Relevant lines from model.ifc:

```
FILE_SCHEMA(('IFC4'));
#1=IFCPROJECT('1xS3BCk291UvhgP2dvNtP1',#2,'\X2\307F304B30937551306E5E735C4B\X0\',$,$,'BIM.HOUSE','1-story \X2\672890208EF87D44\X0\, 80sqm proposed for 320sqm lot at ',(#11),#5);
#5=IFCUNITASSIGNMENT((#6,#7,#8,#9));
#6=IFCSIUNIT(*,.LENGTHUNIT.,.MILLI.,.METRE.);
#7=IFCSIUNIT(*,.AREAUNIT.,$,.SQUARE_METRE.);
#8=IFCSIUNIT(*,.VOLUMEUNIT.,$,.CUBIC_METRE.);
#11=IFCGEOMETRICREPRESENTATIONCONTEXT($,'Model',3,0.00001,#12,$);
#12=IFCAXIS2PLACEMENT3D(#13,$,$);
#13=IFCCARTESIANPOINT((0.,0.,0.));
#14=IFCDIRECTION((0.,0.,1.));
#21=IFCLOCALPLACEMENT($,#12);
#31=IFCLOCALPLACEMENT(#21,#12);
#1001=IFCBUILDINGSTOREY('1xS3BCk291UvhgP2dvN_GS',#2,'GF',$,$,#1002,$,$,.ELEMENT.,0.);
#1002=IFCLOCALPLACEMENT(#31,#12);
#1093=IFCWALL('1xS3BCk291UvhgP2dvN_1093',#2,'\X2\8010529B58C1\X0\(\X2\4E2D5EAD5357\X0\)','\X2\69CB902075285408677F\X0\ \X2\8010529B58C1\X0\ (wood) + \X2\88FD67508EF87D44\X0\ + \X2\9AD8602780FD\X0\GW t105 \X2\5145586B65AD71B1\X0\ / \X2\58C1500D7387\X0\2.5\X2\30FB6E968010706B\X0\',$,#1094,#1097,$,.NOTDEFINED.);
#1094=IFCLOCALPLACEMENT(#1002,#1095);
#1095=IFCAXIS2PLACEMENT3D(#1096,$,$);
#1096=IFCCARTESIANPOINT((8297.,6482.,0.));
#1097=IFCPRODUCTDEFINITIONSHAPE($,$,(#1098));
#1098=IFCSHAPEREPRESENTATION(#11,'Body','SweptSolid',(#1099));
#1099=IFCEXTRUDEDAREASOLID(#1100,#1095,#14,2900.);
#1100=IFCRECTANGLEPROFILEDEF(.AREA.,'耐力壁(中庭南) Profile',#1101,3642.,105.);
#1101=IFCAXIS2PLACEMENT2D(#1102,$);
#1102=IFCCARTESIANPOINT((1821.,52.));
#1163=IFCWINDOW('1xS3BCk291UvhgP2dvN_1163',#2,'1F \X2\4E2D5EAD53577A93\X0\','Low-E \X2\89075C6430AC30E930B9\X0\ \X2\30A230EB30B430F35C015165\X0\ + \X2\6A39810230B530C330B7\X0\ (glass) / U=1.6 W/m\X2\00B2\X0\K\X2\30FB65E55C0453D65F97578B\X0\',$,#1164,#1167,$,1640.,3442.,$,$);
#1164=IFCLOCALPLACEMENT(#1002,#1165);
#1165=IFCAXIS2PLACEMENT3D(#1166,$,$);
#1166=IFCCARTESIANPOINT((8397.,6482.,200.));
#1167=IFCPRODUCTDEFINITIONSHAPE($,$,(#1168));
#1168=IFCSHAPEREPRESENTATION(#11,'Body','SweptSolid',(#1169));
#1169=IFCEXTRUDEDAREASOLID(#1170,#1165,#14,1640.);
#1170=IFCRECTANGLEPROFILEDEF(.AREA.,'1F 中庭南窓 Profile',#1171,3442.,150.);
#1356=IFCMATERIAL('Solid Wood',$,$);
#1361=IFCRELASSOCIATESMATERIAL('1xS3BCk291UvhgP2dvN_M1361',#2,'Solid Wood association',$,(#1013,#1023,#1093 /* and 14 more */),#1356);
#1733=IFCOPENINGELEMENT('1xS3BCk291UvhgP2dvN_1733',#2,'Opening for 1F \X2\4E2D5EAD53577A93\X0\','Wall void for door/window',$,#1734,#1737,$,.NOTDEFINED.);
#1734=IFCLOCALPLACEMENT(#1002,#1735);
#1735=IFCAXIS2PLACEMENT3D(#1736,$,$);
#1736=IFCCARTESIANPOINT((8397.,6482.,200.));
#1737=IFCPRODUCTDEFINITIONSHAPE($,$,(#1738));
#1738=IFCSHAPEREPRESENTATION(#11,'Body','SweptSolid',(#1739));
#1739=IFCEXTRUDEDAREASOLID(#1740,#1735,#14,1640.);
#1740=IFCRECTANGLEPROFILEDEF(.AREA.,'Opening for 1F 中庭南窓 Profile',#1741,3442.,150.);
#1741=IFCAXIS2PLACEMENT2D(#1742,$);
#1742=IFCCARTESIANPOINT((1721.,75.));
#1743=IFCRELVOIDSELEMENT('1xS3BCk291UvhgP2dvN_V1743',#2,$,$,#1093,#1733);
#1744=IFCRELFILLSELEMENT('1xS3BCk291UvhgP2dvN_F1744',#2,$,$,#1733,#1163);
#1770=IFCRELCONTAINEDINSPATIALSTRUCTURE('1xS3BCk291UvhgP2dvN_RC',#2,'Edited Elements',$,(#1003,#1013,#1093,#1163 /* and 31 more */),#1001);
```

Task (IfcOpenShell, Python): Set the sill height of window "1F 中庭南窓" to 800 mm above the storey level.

```python
import numpy as np
import ifcopenshell
import ifcopenshell.api.geometry
import ifcopenshell.geom
import ifcopenshell.util.element
import ifcopenshell.util.placement
import ifcopenshell.util.shape
import ifcopenshell.util.unit

model = ifcopenshell.open("model.ifc")
unit_scale = ifcopenshell.util.unit.calculate_unit_scale(model)

window = model.by_id(1163)
opening = window.FillsVoids[0].RelatingOpeningElement
storey = ifcopenshell.util.element.get_container(window, ifc_class="IfcBuildingStorey")
level = ifcopenshell.util.placement.get_local_placement(storey.ObjectPlacement)[2, 3]

# The opening's origin need not be at the sill, so measure its lowest point.
shape = ifcopenshell.geom.create_shape(ifcopenshell.geom.settings(), opening)
bottom = ifcopenshell.util.shape.get_shape_bottom_elevation(shape, shape.geometry) / unit_scale
dz = level + 800.0 - bottom

shift = np.array([0.0, 0.0, dz])
# The window is not placed relative to its opening, so move both.
for product in (opening, window):
    matrix = ifcopenshell.util.placement.get_local_placement(product.ObjectPlacement)
    matrix[:3, 3] += shift
    ifcopenshell.api.geometry.edit_object_placement(model, product=product, matrix=matrix, is_si=False)

print(f"moved by {dz * unit_scale:+.3f} m")

model.write("model_rev.ifc")
```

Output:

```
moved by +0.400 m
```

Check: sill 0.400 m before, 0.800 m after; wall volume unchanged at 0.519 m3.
